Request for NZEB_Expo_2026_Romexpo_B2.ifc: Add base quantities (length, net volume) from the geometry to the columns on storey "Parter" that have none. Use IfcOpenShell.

First a look at what the model holds.

```python
import ifcopenshell
import ifcopenshell.util.element
import ifcopenshell.util.unit

model = ifcopenshell.open("NZEB_Expo_2026_Romexpo_B2.ifc")
print(model.schema)
for unit_type in ("LENGTHUNIT", "AREAUNIT", "VOLUMEUNIT"):
    print(unit_type, ifcopenshell.util.unit.calculate_unit_scale(model, unit_type))
storey = next(s for s in model.by_type("IfcBuildingStorey") if s.Name == "Parter")
columns = [e for e in ifcopenshell.util.element.get_decomposition(storey) if e.is_a("IfcColumn")]
for e in sorted(columns, key=lambda e: e.id()):
    print(e.id(), e.is_a(), e.Name, list(ifcopenshell.util.element.get_psets(e, qtos_only=True)), sep=" | ")
```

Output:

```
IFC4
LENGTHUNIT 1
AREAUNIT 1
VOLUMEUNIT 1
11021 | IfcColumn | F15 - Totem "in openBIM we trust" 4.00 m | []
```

```python
import ifcopenshell
import ifcopenshell.api.pset
import ifcopenshell.geom
import ifcopenshell.util.element
import ifcopenshell.util.shape
import ifcopenshell.util.unit

model = ifcopenshell.open("NZEB_Expo_2026_Romexpo_B2.ifc")
unit_scale = ifcopenshell.util.unit.calculate_unit_scale(model)
volume_scale = ifcopenshell.util.unit.calculate_unit_scale(model, "VOLUMEUNIT")
settings = ifcopenshell.geom.settings()

storey = next(s for s in model.by_type("IfcBuildingStorey") if s.Name == "Parter")
columns = [e for e in ifcopenshell.util.element.get_decomposition(storey) if e.is_a("IfcColumn")]

for e in sorted(columns, key=lambda e: e.id()):
    if ifcopenshell.util.element.get_psets(e, qtos_only=True, should_inherit=False):
        continue
    # Geometry comes back in metres, in the element's own axes.
    shape = ifcopenshell.geom.create_shape(settings, e)
    values = {
        "Length": ifcopenshell.util.shape.get_z(shape.geometry) / unit_scale,
        "NetVolume": ifcopenshell.util.shape.get_volume(shape.geometry) / volume_scale,
    }
    qto = ifcopenshell.api.pset.add_qto(model, product=e, name="Qto_ColumnBaseQuantities")
    ifcopenshell.api.pset.edit_qto(model, qto=qto, properties=values)
    print(e.id(), {k: round(v, 3) for k, v in values.items()})

model.write("NZEB_Expo_2026_Romexpo_B2_edited.ifc")
```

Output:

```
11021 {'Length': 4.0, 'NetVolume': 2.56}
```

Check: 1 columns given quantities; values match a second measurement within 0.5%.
